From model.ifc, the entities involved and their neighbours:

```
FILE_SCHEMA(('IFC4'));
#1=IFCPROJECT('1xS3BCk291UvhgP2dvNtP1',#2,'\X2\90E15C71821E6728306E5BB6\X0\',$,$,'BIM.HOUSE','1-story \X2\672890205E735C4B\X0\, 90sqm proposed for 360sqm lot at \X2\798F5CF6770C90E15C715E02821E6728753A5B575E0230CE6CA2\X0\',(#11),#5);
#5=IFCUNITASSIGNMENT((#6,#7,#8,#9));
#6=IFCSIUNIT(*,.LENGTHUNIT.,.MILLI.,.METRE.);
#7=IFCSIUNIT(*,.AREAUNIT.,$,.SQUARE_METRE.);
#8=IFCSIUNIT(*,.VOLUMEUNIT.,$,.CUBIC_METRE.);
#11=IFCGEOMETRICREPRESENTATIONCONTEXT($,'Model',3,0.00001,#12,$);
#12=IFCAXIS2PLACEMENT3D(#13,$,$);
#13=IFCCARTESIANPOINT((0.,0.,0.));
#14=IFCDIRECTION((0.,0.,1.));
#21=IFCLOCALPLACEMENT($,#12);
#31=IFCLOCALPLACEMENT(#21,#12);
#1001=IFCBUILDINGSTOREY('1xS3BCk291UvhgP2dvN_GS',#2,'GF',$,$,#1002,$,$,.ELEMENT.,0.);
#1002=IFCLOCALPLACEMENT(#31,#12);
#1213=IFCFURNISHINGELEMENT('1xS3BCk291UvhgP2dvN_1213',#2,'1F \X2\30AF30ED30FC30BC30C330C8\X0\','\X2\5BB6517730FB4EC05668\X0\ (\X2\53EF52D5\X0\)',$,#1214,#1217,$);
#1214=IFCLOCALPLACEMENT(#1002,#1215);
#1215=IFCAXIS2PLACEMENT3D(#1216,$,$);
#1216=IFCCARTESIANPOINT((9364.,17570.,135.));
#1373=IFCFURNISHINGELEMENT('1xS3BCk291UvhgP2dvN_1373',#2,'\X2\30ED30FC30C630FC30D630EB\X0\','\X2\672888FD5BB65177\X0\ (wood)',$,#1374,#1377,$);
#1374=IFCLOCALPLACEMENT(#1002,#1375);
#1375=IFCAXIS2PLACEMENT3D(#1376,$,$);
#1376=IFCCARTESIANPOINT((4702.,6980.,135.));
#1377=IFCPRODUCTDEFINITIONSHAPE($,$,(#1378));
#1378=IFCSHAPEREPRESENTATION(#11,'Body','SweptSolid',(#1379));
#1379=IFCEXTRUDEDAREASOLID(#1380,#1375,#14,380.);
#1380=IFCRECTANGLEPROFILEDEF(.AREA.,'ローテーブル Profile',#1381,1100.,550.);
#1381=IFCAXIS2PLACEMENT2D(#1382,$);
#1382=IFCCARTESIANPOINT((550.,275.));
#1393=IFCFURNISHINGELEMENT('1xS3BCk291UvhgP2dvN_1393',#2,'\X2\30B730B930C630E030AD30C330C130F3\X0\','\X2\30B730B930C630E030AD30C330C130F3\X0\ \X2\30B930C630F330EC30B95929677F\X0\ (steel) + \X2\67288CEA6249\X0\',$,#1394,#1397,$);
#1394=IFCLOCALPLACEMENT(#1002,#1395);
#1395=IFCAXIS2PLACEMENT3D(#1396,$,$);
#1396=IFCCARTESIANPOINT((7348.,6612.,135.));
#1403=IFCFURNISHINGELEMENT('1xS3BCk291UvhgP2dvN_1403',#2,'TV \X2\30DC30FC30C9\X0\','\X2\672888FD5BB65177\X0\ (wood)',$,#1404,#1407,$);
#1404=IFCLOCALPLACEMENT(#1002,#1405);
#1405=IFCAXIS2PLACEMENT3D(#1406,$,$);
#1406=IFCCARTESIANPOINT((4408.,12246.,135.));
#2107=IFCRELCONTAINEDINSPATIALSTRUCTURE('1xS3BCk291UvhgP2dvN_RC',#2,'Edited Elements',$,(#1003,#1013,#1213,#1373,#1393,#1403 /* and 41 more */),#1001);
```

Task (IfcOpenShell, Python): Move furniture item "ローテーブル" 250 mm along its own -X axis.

```python
import ifcopenshell
import ifcopenshell.api.geometry
import ifcopenshell.util.placement
import ifcopenshell.util.unit

model = ifcopenshell.open("model.ifc")
unit_scale = ifcopenshell.util.unit.calculate_unit_scale(model)

item = model.by_id(1373)
matrix = ifcopenshell.util.placement.get_local_placement(item.ObjectPlacement)
matrix[:3, 3] -= matrix[:3, 0] * 0.25 / unit_scale
ifcopenshell.api.geometry.edit_object_placement(model, product=item, matrix=matrix, is_si=False)

print(ifcopenshell.util.placement.get_local_placement(item.ObjectPlacement).round(3) + 0.0)

model.write("model_v2.ifc")
```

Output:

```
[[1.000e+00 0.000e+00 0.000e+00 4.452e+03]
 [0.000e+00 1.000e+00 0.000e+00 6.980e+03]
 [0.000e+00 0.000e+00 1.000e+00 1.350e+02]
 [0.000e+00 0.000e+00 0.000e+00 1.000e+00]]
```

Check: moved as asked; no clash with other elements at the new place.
